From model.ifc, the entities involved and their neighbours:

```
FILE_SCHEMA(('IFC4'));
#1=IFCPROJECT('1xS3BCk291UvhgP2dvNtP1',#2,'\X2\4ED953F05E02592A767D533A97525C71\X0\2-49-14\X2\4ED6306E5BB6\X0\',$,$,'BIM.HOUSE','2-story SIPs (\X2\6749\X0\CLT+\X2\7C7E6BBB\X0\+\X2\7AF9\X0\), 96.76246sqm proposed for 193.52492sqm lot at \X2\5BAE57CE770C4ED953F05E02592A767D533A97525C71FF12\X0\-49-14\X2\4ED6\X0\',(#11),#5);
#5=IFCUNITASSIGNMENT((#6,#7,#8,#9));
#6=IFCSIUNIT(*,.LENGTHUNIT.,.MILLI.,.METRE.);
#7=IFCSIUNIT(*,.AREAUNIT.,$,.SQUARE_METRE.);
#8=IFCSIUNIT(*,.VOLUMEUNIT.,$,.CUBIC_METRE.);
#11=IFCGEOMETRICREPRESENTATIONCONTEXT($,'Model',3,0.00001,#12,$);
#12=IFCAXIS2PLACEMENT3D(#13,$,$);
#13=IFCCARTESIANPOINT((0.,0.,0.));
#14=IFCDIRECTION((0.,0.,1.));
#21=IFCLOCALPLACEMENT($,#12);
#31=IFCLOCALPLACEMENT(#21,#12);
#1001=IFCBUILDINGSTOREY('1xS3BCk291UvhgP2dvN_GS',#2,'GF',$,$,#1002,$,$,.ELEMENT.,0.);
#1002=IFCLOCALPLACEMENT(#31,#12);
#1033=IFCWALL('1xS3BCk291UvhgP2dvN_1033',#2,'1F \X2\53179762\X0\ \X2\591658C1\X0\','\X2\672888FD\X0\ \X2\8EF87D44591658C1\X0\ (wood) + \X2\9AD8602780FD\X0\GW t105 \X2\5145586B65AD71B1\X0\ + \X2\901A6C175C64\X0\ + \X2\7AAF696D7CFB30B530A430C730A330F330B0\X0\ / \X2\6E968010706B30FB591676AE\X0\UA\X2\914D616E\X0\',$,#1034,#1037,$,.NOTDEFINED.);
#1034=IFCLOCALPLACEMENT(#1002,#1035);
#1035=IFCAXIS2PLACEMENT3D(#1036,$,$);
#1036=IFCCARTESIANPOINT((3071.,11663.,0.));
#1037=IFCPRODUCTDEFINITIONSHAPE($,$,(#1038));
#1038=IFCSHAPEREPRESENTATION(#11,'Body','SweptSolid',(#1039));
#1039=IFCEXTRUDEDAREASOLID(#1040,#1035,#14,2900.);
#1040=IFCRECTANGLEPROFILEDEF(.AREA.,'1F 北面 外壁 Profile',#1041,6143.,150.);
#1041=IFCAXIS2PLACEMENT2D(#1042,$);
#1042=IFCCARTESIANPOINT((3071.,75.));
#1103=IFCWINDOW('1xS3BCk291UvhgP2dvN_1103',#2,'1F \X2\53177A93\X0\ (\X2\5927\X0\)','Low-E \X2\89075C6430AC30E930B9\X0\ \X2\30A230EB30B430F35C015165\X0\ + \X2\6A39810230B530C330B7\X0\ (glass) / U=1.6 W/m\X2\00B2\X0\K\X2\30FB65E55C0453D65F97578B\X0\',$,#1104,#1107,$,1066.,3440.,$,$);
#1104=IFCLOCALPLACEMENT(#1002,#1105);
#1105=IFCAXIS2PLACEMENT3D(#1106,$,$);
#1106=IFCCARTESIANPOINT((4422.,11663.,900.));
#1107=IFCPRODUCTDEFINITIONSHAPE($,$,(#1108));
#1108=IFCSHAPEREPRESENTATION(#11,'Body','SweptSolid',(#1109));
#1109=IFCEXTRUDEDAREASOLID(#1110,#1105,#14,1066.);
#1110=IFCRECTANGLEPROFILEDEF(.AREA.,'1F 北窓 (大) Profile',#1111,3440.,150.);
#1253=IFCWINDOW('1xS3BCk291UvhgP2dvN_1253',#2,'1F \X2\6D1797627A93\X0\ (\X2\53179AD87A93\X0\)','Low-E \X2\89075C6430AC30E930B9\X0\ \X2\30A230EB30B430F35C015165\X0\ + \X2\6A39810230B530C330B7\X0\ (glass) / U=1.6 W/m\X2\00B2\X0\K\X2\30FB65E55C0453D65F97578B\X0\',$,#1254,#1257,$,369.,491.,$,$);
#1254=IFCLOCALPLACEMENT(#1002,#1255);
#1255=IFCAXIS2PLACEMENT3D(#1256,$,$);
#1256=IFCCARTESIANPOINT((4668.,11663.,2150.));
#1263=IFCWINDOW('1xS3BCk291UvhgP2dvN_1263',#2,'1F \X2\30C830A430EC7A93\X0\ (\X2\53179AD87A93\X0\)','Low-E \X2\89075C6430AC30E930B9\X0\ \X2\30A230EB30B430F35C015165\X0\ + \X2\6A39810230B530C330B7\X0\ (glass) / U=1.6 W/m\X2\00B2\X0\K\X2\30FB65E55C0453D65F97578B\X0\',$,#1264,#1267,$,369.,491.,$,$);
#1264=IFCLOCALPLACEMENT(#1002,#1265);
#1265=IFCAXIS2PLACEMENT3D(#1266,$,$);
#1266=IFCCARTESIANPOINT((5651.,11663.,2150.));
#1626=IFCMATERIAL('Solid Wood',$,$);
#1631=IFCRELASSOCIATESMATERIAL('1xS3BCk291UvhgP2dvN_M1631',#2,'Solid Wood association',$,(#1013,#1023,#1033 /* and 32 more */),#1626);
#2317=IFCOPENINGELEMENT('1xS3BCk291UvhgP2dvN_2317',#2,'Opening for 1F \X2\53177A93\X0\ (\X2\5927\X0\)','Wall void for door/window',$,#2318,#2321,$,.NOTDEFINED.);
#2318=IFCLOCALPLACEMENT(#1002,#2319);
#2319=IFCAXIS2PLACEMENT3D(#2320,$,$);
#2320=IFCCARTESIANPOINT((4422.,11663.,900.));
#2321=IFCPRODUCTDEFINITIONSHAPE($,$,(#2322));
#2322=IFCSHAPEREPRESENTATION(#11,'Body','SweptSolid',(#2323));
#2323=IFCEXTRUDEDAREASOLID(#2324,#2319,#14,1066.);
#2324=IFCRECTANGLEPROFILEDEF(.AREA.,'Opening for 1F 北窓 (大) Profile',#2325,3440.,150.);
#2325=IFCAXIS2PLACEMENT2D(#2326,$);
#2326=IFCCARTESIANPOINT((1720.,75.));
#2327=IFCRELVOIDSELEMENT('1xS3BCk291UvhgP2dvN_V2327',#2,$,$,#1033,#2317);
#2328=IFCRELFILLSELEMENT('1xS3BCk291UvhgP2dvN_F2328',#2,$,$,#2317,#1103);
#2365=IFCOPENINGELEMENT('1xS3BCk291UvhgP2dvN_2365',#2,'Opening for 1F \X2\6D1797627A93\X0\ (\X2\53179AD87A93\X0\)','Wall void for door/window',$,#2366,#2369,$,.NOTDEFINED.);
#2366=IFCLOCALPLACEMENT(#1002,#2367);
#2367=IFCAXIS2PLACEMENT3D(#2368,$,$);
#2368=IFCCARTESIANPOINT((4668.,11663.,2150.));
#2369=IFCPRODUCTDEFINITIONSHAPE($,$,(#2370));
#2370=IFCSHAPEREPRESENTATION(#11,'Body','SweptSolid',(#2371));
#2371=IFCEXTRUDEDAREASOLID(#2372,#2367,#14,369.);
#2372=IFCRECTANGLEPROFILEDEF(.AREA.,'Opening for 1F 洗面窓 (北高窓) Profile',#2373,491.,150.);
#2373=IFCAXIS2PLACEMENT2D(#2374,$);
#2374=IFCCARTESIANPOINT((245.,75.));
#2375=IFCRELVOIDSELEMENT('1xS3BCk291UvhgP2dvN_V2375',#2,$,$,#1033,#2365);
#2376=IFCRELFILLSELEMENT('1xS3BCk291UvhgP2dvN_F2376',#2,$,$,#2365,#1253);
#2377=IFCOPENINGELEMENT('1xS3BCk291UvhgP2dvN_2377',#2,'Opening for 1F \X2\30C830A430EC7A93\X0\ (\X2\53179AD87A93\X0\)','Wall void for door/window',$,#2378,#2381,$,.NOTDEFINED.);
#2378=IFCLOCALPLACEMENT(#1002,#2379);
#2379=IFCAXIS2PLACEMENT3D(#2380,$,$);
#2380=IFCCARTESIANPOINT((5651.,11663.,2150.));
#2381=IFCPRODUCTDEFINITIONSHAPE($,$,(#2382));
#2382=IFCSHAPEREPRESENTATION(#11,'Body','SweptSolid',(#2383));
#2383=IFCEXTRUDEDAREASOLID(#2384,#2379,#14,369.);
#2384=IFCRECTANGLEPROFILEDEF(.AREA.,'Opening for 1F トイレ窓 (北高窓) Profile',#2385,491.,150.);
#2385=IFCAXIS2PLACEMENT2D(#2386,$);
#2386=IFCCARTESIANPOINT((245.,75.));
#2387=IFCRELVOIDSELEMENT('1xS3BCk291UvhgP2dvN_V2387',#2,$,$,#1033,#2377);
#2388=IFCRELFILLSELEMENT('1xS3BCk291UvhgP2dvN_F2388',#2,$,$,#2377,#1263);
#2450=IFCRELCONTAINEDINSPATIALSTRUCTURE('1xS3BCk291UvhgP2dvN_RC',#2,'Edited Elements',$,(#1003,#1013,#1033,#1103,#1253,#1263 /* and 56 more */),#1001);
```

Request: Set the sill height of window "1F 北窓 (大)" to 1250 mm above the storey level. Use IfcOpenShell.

```python
import numpy as np
import ifcopenshell
import ifcopenshell.api.geometry
import ifcopenshell.geom
import ifcopenshell.util.element
import ifcopenshell.util.placement
import ifcopenshell.util.shape
import ifcopenshell.util.unit

model = ifcopenshell.open("model.ifc")
unit_scale = ifcopenshell.util.unit.calculate_unit_scale(model)

window = model.by_id(1103)
opening = window.FillsVoids[0].RelatingOpeningElement
storey = ifcopenshell.util.element.get_container(window, ifc_class="IfcBuildingStorey")
level = ifcopenshell.util.placement.get_local_placement(storey.ObjectPlacement)[2, 3]

# The opening's origin need not be at the sill, so measure its lowest point.
shape = ifcopenshell.geom.create_shape(ifcopenshell.geom.settings(), opening)
bottom = ifcopenshell.util.shape.get_shape_bottom_elevation(shape, shape.geometry) / unit_scale
dz = level + 1.25 / unit_scale - bottom

shift = np.array([0.0, 0.0, dz])
# The window is not placed relative to its opening, so move both.
for product in (opening, window):
    matrix = ifcopenshell.util.placement.get_local_placement(product.ObjectPlacement)
    matrix[:3, 3] += shift
    ifcopenshell.api.geometry.edit_object_placement(model, product=product, matrix=matrix, is_si=False)

print(f"moved by {dz * unit_scale:+.3f} m")

model.write("model-out.ifc")
```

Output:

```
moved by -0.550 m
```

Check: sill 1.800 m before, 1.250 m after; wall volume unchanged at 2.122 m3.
